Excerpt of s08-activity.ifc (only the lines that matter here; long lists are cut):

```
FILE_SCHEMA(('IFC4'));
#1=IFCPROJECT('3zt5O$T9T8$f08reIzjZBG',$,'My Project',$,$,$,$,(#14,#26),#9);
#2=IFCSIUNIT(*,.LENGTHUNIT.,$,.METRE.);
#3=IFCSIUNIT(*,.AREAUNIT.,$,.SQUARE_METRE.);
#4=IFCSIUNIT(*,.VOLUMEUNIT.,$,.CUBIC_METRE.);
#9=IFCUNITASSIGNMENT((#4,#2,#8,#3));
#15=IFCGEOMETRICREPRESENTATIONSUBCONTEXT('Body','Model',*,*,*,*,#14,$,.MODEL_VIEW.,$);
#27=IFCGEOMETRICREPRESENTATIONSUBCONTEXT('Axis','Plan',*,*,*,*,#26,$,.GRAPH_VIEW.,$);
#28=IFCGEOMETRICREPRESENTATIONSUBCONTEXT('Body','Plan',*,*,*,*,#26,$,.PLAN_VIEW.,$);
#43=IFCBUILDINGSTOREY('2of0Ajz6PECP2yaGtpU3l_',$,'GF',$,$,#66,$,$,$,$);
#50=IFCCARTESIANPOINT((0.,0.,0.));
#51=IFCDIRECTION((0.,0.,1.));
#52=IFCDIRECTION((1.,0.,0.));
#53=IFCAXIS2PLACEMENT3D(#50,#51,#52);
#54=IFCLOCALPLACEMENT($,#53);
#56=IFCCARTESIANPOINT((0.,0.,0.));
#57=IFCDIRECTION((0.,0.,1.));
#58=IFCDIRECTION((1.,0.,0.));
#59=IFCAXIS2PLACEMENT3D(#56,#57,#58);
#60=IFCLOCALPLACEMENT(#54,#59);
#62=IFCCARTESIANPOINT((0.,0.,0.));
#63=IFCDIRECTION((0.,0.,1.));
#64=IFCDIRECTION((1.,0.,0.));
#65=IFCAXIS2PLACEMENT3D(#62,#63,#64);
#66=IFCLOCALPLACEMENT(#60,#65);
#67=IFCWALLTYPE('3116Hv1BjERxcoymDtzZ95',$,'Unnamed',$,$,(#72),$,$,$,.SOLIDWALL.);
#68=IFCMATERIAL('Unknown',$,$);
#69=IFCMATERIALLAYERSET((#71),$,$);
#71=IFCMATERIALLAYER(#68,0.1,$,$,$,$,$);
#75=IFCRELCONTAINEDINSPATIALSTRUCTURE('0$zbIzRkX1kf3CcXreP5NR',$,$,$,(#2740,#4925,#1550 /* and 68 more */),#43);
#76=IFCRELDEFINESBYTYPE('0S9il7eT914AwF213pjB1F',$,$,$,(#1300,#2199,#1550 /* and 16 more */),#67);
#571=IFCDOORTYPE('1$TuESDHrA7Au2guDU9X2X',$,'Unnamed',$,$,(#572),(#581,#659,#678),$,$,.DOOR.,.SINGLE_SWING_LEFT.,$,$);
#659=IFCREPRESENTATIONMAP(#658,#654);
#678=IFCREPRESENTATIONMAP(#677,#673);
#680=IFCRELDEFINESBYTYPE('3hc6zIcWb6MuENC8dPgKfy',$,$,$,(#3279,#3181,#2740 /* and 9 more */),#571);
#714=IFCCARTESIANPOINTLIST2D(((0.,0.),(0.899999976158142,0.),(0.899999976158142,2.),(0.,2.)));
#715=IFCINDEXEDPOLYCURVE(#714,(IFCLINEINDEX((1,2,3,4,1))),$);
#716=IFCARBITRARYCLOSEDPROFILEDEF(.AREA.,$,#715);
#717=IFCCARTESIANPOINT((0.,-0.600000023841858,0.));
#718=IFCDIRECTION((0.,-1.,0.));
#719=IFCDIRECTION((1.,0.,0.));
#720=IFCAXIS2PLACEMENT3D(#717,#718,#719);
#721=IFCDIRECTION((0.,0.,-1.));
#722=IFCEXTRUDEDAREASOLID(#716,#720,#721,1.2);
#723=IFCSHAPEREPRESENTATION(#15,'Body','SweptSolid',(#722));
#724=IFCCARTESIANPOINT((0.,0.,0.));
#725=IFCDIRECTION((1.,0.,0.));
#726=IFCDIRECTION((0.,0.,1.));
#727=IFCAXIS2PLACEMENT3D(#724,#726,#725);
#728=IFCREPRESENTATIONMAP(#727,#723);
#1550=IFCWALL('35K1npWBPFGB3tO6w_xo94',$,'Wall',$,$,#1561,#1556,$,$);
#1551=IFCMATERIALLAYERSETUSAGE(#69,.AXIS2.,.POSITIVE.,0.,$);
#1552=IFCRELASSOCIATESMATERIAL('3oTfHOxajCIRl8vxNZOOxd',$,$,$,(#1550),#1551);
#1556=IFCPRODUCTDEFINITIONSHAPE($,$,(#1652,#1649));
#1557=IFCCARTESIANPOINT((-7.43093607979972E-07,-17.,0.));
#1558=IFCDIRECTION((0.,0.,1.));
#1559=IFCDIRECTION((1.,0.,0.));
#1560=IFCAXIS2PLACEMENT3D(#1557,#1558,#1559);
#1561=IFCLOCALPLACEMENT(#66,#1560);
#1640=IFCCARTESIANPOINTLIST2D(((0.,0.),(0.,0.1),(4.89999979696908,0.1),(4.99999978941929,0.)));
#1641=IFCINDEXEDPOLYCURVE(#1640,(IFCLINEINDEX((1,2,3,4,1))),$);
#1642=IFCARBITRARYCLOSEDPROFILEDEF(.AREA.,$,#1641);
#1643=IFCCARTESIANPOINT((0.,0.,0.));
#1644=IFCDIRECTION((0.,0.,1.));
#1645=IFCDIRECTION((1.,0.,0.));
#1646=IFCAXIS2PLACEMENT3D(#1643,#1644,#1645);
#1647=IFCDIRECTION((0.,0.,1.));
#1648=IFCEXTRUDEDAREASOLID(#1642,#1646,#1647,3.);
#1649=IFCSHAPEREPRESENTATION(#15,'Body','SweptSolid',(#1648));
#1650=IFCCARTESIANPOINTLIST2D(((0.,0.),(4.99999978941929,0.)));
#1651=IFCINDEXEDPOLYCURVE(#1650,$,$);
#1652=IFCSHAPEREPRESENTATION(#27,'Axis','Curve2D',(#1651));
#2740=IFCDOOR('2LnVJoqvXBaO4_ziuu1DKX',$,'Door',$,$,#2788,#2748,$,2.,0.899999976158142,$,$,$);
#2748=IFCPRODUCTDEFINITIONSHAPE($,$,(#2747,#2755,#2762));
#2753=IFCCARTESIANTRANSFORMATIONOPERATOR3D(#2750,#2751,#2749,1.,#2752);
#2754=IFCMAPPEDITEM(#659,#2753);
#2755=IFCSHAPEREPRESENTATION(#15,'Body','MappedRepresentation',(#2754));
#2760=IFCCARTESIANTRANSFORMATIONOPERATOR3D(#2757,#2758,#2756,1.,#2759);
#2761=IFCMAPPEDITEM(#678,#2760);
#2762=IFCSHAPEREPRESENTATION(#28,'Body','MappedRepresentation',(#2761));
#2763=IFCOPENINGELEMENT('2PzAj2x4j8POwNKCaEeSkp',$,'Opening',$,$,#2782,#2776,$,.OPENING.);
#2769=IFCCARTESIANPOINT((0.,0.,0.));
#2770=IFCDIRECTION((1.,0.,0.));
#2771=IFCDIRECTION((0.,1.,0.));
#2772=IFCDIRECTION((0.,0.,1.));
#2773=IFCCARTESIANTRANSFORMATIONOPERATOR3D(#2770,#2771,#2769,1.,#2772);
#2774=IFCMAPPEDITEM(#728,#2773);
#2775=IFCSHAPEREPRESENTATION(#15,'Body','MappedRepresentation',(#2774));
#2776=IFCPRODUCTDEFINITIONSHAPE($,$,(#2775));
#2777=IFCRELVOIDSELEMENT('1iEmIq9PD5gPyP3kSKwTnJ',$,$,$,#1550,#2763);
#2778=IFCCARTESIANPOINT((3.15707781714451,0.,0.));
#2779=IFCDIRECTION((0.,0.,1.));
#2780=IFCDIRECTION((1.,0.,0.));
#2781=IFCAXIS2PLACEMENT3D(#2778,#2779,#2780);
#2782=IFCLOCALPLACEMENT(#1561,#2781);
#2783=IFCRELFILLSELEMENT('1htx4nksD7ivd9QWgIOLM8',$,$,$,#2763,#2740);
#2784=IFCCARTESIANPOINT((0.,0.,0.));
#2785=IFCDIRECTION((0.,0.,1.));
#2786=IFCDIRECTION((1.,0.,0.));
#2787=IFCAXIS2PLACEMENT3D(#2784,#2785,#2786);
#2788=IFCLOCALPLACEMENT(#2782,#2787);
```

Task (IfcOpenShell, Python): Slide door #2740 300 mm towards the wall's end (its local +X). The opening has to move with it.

```python
import ifcopenshell
import ifcopenshell.api.geometry
import ifcopenshell.util.placement
import ifcopenshell.util.unit

model = ifcopenshell.open("s08-activity.ifc")
unit_scale = ifcopenshell.util.unit.calculate_unit_scale(model)

door = model.by_guid("2LnVJoqvXBaO4_ziuu1DKX")
opening = door.FillsVoids[0].RelatingOpeningElement
wall = opening.VoidsElements[0].RelatingBuildingElement

wall_matrix = ifcopenshell.util.placement.get_local_placement(wall.ObjectPlacement)
shift = wall_matrix[:3, 0] * 0.3 / unit_scale
before = ifcopenshell.util.placement.get_local_placement(door.ObjectPlacement)[:3, 3].copy()

# The door is placed relative to its opening, so it follows when the opening moves.
matrix = ifcopenshell.util.placement.get_local_placement(opening.ObjectPlacement)
matrix[:3, 3] += shift
ifcopenshell.api.geometry.edit_object_placement(
    model, product=opening, matrix=matrix, is_si=False, should_transform_children=True
)

after = ifcopenshell.util.placement.get_local_placement(door.ObjectPlacement)[:3, 3]
print("door moved by", (after - before).round(3) + 0.0)

model.write("s08-activity-out.ifc")
```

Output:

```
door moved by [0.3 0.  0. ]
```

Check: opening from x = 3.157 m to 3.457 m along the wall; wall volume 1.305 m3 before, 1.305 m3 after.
